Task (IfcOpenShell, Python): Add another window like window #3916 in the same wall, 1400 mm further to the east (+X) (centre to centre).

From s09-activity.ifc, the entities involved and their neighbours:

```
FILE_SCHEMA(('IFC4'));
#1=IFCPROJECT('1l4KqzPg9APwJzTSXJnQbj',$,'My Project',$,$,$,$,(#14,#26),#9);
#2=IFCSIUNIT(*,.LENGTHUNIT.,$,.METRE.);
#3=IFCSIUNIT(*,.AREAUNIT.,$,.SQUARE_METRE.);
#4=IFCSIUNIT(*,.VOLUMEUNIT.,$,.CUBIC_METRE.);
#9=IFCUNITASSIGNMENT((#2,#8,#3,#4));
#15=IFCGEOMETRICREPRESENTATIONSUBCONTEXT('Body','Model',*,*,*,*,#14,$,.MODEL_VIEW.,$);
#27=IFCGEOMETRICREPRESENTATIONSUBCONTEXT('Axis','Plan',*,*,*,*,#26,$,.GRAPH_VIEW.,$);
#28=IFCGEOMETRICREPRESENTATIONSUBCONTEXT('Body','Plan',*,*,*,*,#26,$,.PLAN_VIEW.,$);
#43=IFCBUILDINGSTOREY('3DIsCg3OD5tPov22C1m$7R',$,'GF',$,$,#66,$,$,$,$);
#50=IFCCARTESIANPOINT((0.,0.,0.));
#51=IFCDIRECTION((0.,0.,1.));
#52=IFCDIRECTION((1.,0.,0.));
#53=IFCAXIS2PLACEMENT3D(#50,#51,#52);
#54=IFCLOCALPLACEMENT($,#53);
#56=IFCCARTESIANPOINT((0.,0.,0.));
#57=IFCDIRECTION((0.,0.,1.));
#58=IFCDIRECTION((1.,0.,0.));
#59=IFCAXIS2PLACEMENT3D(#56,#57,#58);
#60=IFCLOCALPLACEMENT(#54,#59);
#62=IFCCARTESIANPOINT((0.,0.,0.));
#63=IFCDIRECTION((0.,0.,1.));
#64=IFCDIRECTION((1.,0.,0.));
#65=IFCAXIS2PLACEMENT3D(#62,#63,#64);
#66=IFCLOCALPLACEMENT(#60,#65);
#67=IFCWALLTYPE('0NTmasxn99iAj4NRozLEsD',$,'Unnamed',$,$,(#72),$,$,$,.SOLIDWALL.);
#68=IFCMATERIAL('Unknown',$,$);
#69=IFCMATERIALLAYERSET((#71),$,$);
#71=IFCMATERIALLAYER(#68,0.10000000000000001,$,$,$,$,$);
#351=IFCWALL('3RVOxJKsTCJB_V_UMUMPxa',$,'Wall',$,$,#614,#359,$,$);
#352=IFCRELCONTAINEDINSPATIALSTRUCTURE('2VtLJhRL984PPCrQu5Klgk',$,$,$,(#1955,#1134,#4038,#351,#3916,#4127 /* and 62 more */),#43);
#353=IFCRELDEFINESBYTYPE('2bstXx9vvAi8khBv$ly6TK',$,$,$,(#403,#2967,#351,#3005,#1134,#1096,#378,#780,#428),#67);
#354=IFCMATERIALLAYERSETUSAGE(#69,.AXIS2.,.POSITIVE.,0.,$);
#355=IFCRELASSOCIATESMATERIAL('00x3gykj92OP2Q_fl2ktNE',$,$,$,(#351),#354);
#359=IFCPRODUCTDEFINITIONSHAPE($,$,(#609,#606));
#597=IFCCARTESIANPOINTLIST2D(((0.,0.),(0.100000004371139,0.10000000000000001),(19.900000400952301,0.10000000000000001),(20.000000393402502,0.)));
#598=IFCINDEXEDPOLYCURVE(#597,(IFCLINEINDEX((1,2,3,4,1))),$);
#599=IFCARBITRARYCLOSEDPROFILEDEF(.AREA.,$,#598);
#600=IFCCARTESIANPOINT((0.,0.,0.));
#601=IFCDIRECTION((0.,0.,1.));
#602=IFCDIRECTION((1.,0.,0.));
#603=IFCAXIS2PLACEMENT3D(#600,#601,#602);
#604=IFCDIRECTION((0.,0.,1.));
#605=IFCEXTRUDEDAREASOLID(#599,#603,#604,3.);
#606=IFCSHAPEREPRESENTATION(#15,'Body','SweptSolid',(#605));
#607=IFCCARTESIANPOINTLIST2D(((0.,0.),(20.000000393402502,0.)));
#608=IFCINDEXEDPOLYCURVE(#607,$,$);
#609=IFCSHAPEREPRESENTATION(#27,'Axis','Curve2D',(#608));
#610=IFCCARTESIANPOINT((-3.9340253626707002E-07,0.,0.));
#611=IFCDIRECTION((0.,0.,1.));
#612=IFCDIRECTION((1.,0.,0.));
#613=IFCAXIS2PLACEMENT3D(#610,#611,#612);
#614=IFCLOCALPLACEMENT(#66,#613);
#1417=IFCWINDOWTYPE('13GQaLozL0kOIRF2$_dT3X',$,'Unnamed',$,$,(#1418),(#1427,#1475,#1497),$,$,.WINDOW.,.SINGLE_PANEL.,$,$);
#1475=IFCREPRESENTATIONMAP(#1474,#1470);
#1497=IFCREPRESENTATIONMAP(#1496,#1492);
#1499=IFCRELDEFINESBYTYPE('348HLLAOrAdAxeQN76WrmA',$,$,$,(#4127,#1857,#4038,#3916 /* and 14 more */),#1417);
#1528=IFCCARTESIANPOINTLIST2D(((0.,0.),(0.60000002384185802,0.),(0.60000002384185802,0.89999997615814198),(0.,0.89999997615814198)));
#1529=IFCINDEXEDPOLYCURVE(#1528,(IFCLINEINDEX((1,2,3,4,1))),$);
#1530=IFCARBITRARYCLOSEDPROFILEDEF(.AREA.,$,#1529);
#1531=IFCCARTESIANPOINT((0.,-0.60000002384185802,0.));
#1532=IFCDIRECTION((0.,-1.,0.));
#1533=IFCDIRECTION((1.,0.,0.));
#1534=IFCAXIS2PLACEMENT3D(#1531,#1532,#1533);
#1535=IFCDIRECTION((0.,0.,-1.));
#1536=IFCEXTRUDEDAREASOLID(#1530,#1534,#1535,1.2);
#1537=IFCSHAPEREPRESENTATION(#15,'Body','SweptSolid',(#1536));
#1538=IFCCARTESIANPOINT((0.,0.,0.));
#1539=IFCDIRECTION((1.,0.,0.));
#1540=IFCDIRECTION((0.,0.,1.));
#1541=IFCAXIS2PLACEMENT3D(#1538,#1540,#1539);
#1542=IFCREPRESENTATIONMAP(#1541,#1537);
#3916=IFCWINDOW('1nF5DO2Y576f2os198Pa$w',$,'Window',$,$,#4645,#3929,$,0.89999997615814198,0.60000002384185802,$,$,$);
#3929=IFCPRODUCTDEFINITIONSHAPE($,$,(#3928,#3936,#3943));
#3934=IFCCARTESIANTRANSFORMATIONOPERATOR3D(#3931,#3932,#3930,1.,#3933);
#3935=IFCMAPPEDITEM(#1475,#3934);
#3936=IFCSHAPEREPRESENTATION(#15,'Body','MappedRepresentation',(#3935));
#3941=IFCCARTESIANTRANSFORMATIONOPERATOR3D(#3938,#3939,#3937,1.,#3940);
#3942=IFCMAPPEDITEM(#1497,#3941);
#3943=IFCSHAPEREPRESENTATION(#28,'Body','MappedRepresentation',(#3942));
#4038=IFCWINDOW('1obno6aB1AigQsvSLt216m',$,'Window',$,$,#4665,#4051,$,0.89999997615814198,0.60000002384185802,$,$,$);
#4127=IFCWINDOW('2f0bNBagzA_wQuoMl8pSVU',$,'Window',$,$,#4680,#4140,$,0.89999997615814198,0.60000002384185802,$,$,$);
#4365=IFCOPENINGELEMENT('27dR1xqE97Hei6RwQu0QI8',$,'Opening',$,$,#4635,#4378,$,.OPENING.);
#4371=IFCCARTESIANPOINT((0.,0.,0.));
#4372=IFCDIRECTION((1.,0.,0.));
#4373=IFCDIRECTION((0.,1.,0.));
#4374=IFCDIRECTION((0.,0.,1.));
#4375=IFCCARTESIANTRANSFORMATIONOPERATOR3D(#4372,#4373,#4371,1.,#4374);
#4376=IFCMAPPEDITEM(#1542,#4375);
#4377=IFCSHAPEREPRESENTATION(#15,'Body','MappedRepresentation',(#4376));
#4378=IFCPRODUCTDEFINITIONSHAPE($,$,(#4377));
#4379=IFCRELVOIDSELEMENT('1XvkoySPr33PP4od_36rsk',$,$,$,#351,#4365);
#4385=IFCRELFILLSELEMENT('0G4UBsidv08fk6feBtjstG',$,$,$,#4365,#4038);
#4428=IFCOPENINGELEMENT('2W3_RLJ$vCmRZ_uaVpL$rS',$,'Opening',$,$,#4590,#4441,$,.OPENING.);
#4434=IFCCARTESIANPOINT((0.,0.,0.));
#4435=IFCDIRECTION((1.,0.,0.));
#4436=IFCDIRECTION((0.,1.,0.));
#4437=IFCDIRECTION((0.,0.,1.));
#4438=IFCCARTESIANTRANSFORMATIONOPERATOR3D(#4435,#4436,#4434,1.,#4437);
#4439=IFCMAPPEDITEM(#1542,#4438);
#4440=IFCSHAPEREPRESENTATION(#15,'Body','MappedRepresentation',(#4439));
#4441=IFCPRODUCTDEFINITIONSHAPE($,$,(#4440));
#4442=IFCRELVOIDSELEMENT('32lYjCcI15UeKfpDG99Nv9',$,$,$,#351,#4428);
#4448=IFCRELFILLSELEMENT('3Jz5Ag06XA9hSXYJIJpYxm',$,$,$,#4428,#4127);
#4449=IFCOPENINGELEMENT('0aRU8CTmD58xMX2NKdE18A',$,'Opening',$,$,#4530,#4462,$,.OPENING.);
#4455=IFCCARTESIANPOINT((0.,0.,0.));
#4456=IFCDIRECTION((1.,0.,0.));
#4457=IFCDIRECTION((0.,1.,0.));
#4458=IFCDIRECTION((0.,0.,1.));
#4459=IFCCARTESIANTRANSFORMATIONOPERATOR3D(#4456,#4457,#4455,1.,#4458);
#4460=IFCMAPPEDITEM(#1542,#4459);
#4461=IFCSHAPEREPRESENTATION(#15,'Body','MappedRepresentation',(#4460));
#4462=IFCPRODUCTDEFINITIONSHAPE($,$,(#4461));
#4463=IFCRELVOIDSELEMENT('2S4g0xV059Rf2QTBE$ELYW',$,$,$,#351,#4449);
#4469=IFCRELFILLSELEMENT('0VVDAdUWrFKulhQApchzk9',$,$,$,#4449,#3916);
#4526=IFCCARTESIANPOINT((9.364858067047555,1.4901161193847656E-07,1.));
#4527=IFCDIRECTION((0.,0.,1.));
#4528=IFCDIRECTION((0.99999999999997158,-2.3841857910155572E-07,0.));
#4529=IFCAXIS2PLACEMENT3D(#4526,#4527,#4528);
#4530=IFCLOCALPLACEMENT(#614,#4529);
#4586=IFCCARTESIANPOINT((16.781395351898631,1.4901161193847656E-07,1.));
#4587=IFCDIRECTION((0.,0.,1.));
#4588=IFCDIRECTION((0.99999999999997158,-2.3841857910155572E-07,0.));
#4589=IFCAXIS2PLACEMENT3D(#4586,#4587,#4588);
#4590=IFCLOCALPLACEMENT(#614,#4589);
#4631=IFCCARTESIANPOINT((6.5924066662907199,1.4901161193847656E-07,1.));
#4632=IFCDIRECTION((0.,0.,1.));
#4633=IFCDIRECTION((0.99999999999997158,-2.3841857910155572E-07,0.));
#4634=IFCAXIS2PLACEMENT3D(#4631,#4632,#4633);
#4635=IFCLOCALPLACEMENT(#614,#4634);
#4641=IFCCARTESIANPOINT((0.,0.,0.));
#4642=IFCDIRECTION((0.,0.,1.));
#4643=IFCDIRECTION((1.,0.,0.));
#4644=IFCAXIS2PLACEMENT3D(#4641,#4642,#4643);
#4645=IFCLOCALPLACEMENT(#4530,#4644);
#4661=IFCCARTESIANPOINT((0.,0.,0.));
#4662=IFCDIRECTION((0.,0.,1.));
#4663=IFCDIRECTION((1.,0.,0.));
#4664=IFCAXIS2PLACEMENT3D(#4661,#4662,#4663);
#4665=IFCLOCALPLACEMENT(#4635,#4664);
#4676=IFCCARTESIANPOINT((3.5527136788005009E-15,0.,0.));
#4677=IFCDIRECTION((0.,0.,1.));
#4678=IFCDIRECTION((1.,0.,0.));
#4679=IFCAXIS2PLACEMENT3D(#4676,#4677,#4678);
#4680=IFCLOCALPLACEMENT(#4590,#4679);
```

```python
import ifcopenshell
import ifcopenshell.api.feature
import ifcopenshell.api.geometry
import ifcopenshell.api.root
import ifcopenshell.geom
import ifcopenshell.util.element
import ifcopenshell.util.placement
import ifcopenshell.util.shape
import ifcopenshell.util.unit

model = ifcopenshell.open("s09-activity.ifc")
unit_scale = ifcopenshell.util.unit.calculate_unit_scale(model)
settings = ifcopenshell.geom.settings()


def volume(element):
    """Net volume in cubic metres, openings subtracted."""
    shape = ifcopenshell.geom.create_shape(settings, element)
    return ifcopenshell.util.shape.get_volume(shape.geometry)


window = model.by_guid("1nF5DO2Y576f2os198Pa$w")
opening = window.FillsVoids[0].RelatingOpeningElement
wall = opening.VoidsElements[0].RelatingBuildingElement
before = volume(wall)
shift = ifcopenshell.util.placement.get_local_placement(wall.ObjectPlacement)[:3, 0] * 1.4 / unit_scale

# copy_class copies the void relationship, type, container and properties, but no geometry.
new_opening = ifcopenshell.api.root.copy_class(model, product=opening)
new_opening.Representation = ifcopenshell.util.element.copy_deep(
    model, opening.Representation, exclude=["IfcGeometricRepresentationContext", "IfcRepresentationMap"]
)
new_window = ifcopenshell.api.root.copy_class(model, product=window)
new_window.Representation = ifcopenshell.util.element.copy_deep(
    model, window.Representation, exclude=["IfcGeometricRepresentationContext", "IfcRepresentationMap"]
)
ifcopenshell.api.feature.add_filling(model, opening=new_opening, element=new_window)

for old, new in ((opening, new_opening), (window, new_window)):
    matrix = ifcopenshell.util.placement.get_local_placement(old.ObjectPlacement)
    matrix[:3, 3] += shift
    ifcopenshell.api.geometry.edit_object_placement(model, product=new, matrix=matrix, is_si=False)

after = volume(wall)

print(f"wall volume {before:.3f} -> {after:.3f} m3")

model.write("s09-activity_rev.ifc")
```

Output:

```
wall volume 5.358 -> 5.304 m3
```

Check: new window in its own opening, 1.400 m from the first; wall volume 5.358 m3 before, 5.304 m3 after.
